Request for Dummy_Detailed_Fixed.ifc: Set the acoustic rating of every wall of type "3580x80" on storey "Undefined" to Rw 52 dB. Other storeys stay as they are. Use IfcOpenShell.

First a look at what the model holds.

```python
import ifcopenshell
import ifcopenshell.util.element

model = ifcopenshell.open("Dummy_Detailed_Fixed.ifc")
print(model.schema)
storey = next(s for s in model.by_type("IfcBuildingStorey") if s.Name == "Undefined")
walls = [e for e in ifcopenshell.util.element.get_decomposition(storey) if e.is_a("IfcWall")]
seen = {}
for e in walls:
    element_type = ifcopenshell.util.element.get_type(e)
    key = (element_type.Name if element_type != e and element_type else None, ifcopenshell.util.element.get_pset(e, "Pset_WallCommon", "AcousticRating"))
    seen[key] = seen.get(key, 0) + 1
for (name, value), count in sorted(seen.items(), key=str):
    print(count, "x", name, "|", value)
```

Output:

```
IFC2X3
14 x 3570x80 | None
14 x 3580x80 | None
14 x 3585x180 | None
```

```python
import ifcopenshell
import ifcopenshell.api.pset
import ifcopenshell.util.element

model = ifcopenshell.open("Dummy_Detailed_Fixed.ifc")

storey = next(s for s in model.by_type("IfcBuildingStorey") if s.Name == "Undefined")
walls = [e for e in ifcopenshell.util.element.get_decomposition(storey) if e.is_a("IfcWall")]

count = 0
for e in walls:
    element_type = ifcopenshell.util.element.get_type(e)
    if element_type in (None, e) or element_type.Name != "3580x80":
        continue
    found = ifcopenshell.util.element.get_pset(e, "Pset_WallCommon", should_inherit=False)
    if found:
        pset = model.by_id(found["id"])
        if len(ifcopenshell.util.element.get_elements_by_pset(pset)) > 1:
            pset = ifcopenshell.api.pset.unshare_pset(model, products=[e], pset=pset)[0]
    else:
        pset = ifcopenshell.api.pset.add_pset(model, product=e, name="Pset_WallCommon")
    ifcopenshell.api.pset.edit_pset(model, pset=pset, properties={"AcousticRating": "Rw 52 dB"})
    count += 1

print(count, "walls updated")

model.write("Dummy_Detailed_Fixed-out.ifc")
```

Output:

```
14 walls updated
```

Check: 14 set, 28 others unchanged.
